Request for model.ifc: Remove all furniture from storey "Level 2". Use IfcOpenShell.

First a look at what the model holds.

```python
import ifcopenshell
import ifcopenshell.util.element

model = ifcopenshell.open("model.ifc")
print(model.schema)
storey = next(s for s in model.by_type("IfcBuildingStorey") if s.Name == "Level 2")
furniture = [e for e in ifcopenshell.util.element.get_decomposition(storey) if e.is_a("IfcFurnishingElement")]
seen = {}
for e in furniture:
    element_type = ifcopenshell.util.element.get_type(e)
    name = element_type.Name if element_type not in (None, e) else None
    seen[name] = seen.get(name, 0) + 1
for name, count in sorted(seen.items(), key=str):
    print(count, "x", name)
```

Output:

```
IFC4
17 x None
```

```python
import ifcopenshell
import ifcopenshell.api.root
import ifcopenshell.util.element

model = ifcopenshell.open("model.ifc")

storey = next(s for s in model.by_type("IfcBuildingStorey") if s.Name == "Level 2")
furniture = [e for e in ifcopenshell.util.element.get_decomposition(storey) if e.is_a("IfcFurnishingElement")]

for e in furniture:
    ifcopenshell.api.root.remove_product(model, product=e)
print(len(furniture), "removed")

model.write("model_edited.ifc")
```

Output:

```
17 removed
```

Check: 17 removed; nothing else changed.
